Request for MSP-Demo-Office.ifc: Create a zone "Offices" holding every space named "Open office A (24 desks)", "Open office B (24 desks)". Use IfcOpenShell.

First a look at what the model holds.

```python
import ifcopenshell

model = ifcopenshell.open("MSP-Demo-Office.ifc")
print(model.schema)
seen = {}
for space in model.by_type("IfcSpace"):
    seen[space.LongName] = seen.get(space.LongName, 0) + 1
for name, count in sorted(seen.items(), key=str):
    print(count, "x", name)
print("zones:", [z.Name for z in model.by_type("IfcZone")][:20])
```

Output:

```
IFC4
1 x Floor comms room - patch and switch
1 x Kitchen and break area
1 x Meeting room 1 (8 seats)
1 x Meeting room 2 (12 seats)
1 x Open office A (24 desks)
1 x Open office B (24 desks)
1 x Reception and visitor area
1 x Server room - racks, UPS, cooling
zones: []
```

```python
import ifcopenshell
import ifcopenshell.api.group
import ifcopenshell.api.root

model = ifcopenshell.open("MSP-Demo-Office.ifc")

names = {"Open office A (24 desks)", "Open office B (24 desks)"}
spaces = [s for s in model.by_type("IfcSpace") if s.LongName in names]

zone = ifcopenshell.api.root.create_entity(model, ifc_class="IfcZone", name="Offices")
ifcopenshell.api.group.assign_group(model, products=spaces, group=zone)
print(len(spaces), "spaces in", zone.Name)

model.write("MSP-Demo-Office-out.ifc")
```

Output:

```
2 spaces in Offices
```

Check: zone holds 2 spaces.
